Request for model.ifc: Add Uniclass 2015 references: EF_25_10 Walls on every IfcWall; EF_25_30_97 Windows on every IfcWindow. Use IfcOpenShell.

First a look at what the model holds.

```python
import ifcopenshell

model = ifcopenshell.open("model.ifc")
print(model.schema)
print("classifications:", [c.Name for c in model.by_type("IfcClassification")])
for ifc_class in ("IfcDoor", "IfcRoof", "IfcStair", "IfcWall", "IfcWindow"):
    print(ifc_class, len(model.by_type(ifc_class)))
```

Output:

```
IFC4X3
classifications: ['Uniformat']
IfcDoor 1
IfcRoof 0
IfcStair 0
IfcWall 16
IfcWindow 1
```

```python
import ifcopenshell
import ifcopenshell.api.classification

model = ifcopenshell.open("model.ifc")

system = ifcopenshell.api.classification.add_classification(model, classification="Uniclass 2015")

codes = {
    "IfcWall": ("EF_25_10", "Walls"),
    "IfcWindow": ("EF_25_30_97", "Windows"),
}
for ifc_class, (code, name) in codes.items():
    products = model.by_type(ifc_class)
    ifcopenshell.api.classification.add_reference(
        model, products=products, classification=system, identification=code, name=name
    )
    print(code, len(products))

model.write("model_updated.ifc")
```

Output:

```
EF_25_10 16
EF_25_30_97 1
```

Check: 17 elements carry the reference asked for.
